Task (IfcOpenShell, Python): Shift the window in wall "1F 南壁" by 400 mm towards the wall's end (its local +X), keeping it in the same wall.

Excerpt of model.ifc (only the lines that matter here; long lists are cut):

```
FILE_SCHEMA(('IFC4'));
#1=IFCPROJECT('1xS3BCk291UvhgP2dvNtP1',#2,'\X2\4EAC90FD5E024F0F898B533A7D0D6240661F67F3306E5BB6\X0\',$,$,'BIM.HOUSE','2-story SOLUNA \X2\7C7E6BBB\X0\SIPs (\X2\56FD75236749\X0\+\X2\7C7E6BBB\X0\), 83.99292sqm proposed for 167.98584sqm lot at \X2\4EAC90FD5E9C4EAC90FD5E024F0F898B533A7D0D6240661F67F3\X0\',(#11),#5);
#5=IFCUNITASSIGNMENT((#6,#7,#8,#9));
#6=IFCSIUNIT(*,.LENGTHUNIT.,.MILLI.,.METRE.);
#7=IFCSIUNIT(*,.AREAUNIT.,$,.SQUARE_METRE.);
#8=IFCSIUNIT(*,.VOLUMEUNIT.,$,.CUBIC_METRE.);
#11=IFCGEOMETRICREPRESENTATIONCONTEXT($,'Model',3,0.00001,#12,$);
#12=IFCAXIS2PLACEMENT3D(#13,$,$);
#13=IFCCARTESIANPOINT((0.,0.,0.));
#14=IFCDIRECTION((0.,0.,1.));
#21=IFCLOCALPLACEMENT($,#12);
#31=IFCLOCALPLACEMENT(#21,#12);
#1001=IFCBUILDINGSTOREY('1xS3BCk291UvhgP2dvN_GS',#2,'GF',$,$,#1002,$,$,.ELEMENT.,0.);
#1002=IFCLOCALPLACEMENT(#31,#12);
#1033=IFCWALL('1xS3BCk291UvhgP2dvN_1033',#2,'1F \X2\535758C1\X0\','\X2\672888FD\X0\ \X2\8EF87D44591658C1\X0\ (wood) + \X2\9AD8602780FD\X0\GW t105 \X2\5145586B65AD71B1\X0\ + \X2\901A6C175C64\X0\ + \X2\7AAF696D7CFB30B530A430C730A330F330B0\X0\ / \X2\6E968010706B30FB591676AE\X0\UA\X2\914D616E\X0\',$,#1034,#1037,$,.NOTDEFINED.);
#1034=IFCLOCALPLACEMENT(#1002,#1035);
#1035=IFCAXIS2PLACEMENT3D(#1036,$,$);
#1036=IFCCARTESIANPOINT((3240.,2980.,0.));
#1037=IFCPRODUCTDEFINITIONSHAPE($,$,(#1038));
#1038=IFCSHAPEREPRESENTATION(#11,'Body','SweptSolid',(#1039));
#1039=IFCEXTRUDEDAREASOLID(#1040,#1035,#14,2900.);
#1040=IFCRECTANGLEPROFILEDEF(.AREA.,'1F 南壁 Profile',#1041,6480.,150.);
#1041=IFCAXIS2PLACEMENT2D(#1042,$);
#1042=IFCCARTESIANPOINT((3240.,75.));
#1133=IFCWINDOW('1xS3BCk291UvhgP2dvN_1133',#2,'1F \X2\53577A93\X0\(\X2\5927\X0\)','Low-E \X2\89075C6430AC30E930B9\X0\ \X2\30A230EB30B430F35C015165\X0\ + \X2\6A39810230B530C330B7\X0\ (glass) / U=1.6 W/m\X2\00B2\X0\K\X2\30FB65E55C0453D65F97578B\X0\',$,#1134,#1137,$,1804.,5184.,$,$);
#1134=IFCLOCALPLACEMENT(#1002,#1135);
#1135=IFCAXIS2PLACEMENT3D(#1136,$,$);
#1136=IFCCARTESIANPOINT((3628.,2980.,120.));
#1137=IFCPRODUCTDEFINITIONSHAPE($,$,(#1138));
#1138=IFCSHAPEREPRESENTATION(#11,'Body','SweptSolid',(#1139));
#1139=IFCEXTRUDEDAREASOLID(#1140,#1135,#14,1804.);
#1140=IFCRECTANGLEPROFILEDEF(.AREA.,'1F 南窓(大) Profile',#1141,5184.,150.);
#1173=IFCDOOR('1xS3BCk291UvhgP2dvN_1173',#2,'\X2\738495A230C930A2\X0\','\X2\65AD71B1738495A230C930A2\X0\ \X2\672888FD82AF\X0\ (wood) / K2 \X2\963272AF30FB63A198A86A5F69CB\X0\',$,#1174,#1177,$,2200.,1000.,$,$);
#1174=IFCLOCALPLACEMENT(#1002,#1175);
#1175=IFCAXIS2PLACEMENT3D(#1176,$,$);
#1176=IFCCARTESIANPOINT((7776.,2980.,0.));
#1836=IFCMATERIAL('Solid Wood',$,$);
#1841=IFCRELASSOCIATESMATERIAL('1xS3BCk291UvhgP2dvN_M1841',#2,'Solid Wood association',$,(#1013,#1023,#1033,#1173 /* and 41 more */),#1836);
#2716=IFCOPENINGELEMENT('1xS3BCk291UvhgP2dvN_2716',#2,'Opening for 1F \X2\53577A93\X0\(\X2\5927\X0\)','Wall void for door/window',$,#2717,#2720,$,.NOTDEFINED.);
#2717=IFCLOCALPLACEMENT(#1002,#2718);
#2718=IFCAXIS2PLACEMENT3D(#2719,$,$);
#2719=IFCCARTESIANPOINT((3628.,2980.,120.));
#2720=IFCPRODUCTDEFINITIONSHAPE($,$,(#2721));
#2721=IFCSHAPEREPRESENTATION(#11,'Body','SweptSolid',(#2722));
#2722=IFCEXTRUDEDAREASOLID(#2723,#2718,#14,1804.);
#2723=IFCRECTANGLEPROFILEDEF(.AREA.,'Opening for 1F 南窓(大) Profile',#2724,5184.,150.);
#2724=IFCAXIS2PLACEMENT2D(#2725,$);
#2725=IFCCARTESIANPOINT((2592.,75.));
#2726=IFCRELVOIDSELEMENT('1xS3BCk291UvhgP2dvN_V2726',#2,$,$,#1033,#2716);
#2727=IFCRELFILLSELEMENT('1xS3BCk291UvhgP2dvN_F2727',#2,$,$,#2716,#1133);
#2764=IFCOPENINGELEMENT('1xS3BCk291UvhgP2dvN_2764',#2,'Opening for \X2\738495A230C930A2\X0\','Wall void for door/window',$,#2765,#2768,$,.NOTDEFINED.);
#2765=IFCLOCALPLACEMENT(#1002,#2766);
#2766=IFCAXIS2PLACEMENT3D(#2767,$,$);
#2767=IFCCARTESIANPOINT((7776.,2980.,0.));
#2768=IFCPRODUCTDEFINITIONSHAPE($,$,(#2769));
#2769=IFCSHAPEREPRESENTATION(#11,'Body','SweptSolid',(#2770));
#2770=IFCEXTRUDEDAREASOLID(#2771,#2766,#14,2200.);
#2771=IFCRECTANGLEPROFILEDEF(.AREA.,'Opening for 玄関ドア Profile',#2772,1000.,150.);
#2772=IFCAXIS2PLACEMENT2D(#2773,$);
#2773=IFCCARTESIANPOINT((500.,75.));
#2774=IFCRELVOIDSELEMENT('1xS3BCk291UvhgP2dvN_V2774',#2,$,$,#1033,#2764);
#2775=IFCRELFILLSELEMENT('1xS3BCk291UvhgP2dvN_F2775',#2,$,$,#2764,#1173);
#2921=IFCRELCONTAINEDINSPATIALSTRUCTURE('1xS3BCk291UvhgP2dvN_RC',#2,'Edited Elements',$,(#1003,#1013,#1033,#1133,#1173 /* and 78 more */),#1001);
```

```python
import ifcopenshell
import ifcopenshell.api.geometry
import ifcopenshell.util.placement
import ifcopenshell.util.unit

model = ifcopenshell.open("model.ifc")
unit_scale = ifcopenshell.util.unit.calculate_unit_scale(model)

window = model.by_guid("1xS3BCk291UvhgP2dvN_1133")
opening = window.FillsVoids[0].RelatingOpeningElement
wall = opening.VoidsElements[0].RelatingBuildingElement

wall_matrix = ifcopenshell.util.placement.get_local_placement(wall.ObjectPlacement)
shift = wall_matrix[:3, 0] * 0.4 / unit_scale
before = ifcopenshell.util.placement.get_local_placement(window.ObjectPlacement)[:3, 3].copy()

# The window is not placed relative to its opening, so move both.
for product in (opening, window):
    matrix = ifcopenshell.util.placement.get_local_placement(product.ObjectPlacement)
    matrix[:3, 3] += shift
    ifcopenshell.api.geometry.edit_object_placement(model, product=product, matrix=matrix, is_si=False)

after = ifcopenshell.util.placement.get_local_placement(window.ObjectPlacement)[:3, 3]
print("window moved by", (after - before).round(3) + 0.0)

model.write("model_rev.ifc")
```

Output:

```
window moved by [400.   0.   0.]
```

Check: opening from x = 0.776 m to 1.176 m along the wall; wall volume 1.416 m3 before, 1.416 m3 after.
